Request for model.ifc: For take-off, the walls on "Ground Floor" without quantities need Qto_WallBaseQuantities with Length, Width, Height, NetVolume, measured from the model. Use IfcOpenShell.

First a look at what the model holds.

```python
import ifcopenshell
import ifcopenshell.util.element
import ifcopenshell.util.unit

model = ifcopenshell.open("model.ifc")
print(model.schema)
for unit_type in ("LENGTHUNIT", "AREAUNIT", "VOLUMEUNIT"):
    print(unit_type, ifcopenshell.util.unit.calculate_unit_scale(model, unit_type))
storey = next(s for s in model.by_type("IfcBuildingStorey") if s.Name == "Ground Floor")
walls = [e for e in ifcopenshell.util.element.get_decomposition(storey) if e.is_a("IfcWall")]
for e in sorted(walls, key=lambda e: e.id()):
    print(e.id(), e.is_a(), e.Name, list(ifcopenshell.util.element.get_psets(e, qtos_only=True)), sep=" | ")
```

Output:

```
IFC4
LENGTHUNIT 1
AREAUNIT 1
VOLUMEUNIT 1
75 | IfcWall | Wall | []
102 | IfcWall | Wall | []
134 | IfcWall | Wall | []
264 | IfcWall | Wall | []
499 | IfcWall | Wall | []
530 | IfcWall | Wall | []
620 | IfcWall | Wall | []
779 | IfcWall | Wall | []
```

```python
import ifcopenshell
import ifcopenshell.api.pset
import ifcopenshell.geom
import ifcopenshell.util.element
import ifcopenshell.util.shape
import ifcopenshell.util.unit

model = ifcopenshell.open("model.ifc")
unit_scale = ifcopenshell.util.unit.calculate_unit_scale(model)
volume_scale = ifcopenshell.util.unit.calculate_unit_scale(model, "VOLUMEUNIT")
settings = ifcopenshell.geom.settings()

storey = next(s for s in model.by_type("IfcBuildingStorey") if s.Name == "Ground Floor")
walls = [e for e in ifcopenshell.util.element.get_decomposition(storey) if e.is_a("IfcWall")]

for e in sorted(walls, key=lambda e: e.id()):
    if ifcopenshell.util.element.get_psets(e, qtos_only=True, should_inherit=False):
        continue
    # Geometry comes back in metres, in the element's own axes.
    shape = ifcopenshell.geom.create_shape(settings, e)
    values = {
        "Length": ifcopenshell.util.shape.get_x(shape.geometry) / unit_scale,
        "Width": ifcopenshell.util.shape.get_y(shape.geometry) / unit_scale,
        "Height": ifcopenshell.util.shape.get_z(shape.geometry) / unit_scale,
        "NetVolume": ifcopenshell.util.shape.get_volume(shape.geometry) / volume_scale,
    }
    qto = ifcopenshell.api.pset.add_qto(model, product=e, name="Qto_WallBaseQuantities")
    ifcopenshell.api.pset.edit_qto(model, qto=qto, properties=values)
    print(e.id(), {k: round(v, 3) for k, v in values.items()})

model.write("model_rev.ifc")
```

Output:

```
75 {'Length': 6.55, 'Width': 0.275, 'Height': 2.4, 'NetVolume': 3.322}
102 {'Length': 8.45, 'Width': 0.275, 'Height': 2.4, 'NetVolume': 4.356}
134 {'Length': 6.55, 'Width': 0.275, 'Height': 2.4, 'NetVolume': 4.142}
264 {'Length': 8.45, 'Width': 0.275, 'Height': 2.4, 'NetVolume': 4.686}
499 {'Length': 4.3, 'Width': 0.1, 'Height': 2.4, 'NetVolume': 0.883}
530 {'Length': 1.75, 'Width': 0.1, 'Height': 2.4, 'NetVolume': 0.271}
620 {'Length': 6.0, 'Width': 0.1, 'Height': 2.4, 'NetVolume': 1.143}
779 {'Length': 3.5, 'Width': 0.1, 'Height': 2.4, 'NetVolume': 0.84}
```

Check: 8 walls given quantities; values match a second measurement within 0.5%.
